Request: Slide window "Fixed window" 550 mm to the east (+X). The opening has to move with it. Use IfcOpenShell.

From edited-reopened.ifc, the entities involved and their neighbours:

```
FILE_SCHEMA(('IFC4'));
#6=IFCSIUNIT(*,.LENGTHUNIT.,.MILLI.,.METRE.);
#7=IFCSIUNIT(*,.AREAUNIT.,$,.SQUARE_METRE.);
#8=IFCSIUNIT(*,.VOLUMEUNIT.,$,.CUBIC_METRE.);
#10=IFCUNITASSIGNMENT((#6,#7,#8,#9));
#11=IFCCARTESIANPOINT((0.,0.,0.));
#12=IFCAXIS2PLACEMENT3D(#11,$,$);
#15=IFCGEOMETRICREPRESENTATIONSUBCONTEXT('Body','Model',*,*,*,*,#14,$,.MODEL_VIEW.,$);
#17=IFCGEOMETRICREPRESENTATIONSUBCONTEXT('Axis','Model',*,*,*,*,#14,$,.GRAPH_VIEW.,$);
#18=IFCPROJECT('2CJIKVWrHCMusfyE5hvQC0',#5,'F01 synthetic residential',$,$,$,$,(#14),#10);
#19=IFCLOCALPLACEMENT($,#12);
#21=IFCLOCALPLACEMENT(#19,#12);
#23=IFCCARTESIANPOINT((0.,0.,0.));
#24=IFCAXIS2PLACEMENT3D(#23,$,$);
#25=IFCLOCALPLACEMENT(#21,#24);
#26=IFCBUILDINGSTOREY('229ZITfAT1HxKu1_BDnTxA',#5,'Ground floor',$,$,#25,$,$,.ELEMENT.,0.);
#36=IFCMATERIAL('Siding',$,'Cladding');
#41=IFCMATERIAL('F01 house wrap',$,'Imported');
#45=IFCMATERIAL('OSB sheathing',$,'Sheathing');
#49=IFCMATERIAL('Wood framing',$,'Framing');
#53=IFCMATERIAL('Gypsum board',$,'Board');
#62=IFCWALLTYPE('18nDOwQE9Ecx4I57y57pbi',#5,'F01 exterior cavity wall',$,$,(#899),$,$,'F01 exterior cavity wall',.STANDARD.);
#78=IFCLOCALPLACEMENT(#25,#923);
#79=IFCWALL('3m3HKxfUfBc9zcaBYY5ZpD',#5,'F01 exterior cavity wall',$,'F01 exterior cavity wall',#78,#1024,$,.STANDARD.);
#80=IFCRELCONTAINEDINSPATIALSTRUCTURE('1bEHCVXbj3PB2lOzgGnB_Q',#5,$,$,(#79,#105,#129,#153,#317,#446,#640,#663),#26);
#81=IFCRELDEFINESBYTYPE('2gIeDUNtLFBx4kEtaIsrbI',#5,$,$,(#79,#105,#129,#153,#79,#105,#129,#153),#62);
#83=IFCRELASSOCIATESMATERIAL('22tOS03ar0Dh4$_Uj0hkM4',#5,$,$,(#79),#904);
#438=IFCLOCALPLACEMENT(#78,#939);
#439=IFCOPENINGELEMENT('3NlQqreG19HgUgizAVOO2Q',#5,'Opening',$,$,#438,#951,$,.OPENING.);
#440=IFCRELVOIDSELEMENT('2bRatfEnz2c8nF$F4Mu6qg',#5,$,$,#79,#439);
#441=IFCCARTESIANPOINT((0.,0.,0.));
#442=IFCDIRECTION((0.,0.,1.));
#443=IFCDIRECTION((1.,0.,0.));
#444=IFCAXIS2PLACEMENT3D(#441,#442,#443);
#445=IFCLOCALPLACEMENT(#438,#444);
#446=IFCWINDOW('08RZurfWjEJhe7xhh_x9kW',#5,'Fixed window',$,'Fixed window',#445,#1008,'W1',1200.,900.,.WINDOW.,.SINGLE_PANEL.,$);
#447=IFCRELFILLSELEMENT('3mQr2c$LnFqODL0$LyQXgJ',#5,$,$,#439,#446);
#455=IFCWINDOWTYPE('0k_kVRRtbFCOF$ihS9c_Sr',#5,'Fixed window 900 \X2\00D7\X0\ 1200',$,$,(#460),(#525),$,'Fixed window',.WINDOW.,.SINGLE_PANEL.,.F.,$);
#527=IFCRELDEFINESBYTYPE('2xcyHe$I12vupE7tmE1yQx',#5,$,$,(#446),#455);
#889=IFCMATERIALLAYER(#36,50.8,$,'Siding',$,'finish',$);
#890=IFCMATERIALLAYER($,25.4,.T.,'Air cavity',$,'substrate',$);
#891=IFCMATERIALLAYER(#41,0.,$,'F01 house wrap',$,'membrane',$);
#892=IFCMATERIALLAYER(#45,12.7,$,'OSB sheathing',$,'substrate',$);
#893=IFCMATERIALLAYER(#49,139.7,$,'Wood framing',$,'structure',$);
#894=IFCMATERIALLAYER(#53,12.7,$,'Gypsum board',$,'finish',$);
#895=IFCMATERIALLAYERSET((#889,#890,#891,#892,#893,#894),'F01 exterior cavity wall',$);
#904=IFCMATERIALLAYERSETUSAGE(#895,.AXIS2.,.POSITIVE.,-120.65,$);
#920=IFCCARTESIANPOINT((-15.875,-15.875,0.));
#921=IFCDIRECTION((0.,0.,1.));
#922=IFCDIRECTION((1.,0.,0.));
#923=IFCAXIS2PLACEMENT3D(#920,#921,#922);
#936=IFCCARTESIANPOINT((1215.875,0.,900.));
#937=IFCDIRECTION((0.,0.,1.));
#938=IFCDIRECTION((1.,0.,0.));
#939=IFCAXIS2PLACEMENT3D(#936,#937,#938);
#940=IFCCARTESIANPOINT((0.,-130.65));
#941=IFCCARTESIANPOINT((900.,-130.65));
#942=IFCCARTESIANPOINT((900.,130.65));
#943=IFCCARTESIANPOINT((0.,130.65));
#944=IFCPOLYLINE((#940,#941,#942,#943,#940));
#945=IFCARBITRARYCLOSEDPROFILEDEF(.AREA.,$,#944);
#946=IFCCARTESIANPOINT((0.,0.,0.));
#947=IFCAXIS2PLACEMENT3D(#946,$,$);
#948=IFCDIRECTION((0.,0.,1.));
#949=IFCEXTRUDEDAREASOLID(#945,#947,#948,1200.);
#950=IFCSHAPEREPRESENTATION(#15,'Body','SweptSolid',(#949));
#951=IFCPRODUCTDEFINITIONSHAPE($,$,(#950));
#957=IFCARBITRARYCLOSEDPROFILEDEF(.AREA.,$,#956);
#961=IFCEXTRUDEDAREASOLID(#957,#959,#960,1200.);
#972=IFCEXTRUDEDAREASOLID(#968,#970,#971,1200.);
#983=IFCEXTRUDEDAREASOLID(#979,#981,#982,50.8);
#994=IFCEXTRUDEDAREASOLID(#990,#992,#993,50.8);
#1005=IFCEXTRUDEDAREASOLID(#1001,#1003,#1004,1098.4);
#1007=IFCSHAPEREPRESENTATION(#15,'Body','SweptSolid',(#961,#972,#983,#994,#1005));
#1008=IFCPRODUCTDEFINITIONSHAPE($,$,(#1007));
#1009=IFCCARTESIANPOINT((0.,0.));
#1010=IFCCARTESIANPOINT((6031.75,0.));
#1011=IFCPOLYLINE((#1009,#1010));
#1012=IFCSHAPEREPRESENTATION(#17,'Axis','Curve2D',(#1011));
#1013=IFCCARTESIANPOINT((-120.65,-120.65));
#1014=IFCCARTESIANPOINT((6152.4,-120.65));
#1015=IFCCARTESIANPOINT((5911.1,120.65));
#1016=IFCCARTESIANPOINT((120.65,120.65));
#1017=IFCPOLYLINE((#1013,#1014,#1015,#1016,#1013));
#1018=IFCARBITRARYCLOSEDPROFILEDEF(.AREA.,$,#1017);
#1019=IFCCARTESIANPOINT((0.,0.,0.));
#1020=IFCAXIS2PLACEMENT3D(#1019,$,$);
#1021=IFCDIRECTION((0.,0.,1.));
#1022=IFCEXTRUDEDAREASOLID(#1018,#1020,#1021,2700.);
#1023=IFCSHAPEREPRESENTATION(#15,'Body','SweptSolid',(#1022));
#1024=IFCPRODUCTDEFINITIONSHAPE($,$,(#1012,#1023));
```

```python
import ifcopenshell
import ifcopenshell.api.geometry
import ifcopenshell.util.placement
import ifcopenshell.util.unit

model = ifcopenshell.open("edited-reopened.ifc")
unit_scale = ifcopenshell.util.unit.calculate_unit_scale(model)

window = model.by_guid("08RZurfWjEJhe7xhh_x9kW")
opening = window.FillsVoids[0].RelatingOpeningElement
wall = opening.VoidsElements[0].RelatingBuildingElement

wall_matrix = ifcopenshell.util.placement.get_local_placement(wall.ObjectPlacement)
shift = wall_matrix[:3, 0] * 0.55 / unit_scale
before = ifcopenshell.util.placement.get_local_placement(window.ObjectPlacement)[:3, 3].copy()

# The window is placed relative to its opening, so it follows when the opening moves.
matrix = ifcopenshell.util.placement.get_local_placement(opening.ObjectPlacement)
matrix[:3, 3] += shift
ifcopenshell.api.geometry.edit_object_placement(
    model, product=opening, matrix=matrix, is_si=False, should_transform_children=True
)

after = ifcopenshell.util.placement.get_local_placement(window.ObjectPlacement)[:3, 3]
print("window moved by", (after - before).round(3) + 0.0)

model.write("edited-reopened_edited.ifc")
```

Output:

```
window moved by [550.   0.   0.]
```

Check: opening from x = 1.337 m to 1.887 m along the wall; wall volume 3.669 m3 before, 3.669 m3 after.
